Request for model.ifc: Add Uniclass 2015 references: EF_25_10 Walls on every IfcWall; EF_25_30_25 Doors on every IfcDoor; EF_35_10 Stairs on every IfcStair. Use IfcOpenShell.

First a look at what the model holds.

```python
import ifcopenshell

model = ifcopenshell.open("model.ifc")
print(model.schema)
print("classifications:", [c.Name for c in model.by_type("IfcClassification")])
for ifc_class in ("IfcDoor", "IfcRoof", "IfcStair", "IfcWall", "IfcWindow"):
    print(ifc_class, len(model.by_type(ifc_class)))
```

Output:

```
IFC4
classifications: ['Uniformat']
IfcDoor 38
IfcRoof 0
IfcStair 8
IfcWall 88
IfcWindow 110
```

```python
import ifcopenshell
import ifcopenshell.api.classification

model = ifcopenshell.open("model.ifc")

system = ifcopenshell.api.classification.add_classification(model, classification="Uniclass 2015")

codes = {
    "IfcWall": ("EF_25_10", "Walls"),
    "IfcDoor": ("EF_25_30_25", "Doors"),
    "IfcStair": ("EF_35_10", "Stairs"),
}
for ifc_class, (code, name) in codes.items():
    products = model.by_type(ifc_class)
    ifcopenshell.api.classification.add_reference(
        model, products=products, classification=system, identification=code, name=name
    )
    print(code, len(products))

model.write("model-out.ifc")
```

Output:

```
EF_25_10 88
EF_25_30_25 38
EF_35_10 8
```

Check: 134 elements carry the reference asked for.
